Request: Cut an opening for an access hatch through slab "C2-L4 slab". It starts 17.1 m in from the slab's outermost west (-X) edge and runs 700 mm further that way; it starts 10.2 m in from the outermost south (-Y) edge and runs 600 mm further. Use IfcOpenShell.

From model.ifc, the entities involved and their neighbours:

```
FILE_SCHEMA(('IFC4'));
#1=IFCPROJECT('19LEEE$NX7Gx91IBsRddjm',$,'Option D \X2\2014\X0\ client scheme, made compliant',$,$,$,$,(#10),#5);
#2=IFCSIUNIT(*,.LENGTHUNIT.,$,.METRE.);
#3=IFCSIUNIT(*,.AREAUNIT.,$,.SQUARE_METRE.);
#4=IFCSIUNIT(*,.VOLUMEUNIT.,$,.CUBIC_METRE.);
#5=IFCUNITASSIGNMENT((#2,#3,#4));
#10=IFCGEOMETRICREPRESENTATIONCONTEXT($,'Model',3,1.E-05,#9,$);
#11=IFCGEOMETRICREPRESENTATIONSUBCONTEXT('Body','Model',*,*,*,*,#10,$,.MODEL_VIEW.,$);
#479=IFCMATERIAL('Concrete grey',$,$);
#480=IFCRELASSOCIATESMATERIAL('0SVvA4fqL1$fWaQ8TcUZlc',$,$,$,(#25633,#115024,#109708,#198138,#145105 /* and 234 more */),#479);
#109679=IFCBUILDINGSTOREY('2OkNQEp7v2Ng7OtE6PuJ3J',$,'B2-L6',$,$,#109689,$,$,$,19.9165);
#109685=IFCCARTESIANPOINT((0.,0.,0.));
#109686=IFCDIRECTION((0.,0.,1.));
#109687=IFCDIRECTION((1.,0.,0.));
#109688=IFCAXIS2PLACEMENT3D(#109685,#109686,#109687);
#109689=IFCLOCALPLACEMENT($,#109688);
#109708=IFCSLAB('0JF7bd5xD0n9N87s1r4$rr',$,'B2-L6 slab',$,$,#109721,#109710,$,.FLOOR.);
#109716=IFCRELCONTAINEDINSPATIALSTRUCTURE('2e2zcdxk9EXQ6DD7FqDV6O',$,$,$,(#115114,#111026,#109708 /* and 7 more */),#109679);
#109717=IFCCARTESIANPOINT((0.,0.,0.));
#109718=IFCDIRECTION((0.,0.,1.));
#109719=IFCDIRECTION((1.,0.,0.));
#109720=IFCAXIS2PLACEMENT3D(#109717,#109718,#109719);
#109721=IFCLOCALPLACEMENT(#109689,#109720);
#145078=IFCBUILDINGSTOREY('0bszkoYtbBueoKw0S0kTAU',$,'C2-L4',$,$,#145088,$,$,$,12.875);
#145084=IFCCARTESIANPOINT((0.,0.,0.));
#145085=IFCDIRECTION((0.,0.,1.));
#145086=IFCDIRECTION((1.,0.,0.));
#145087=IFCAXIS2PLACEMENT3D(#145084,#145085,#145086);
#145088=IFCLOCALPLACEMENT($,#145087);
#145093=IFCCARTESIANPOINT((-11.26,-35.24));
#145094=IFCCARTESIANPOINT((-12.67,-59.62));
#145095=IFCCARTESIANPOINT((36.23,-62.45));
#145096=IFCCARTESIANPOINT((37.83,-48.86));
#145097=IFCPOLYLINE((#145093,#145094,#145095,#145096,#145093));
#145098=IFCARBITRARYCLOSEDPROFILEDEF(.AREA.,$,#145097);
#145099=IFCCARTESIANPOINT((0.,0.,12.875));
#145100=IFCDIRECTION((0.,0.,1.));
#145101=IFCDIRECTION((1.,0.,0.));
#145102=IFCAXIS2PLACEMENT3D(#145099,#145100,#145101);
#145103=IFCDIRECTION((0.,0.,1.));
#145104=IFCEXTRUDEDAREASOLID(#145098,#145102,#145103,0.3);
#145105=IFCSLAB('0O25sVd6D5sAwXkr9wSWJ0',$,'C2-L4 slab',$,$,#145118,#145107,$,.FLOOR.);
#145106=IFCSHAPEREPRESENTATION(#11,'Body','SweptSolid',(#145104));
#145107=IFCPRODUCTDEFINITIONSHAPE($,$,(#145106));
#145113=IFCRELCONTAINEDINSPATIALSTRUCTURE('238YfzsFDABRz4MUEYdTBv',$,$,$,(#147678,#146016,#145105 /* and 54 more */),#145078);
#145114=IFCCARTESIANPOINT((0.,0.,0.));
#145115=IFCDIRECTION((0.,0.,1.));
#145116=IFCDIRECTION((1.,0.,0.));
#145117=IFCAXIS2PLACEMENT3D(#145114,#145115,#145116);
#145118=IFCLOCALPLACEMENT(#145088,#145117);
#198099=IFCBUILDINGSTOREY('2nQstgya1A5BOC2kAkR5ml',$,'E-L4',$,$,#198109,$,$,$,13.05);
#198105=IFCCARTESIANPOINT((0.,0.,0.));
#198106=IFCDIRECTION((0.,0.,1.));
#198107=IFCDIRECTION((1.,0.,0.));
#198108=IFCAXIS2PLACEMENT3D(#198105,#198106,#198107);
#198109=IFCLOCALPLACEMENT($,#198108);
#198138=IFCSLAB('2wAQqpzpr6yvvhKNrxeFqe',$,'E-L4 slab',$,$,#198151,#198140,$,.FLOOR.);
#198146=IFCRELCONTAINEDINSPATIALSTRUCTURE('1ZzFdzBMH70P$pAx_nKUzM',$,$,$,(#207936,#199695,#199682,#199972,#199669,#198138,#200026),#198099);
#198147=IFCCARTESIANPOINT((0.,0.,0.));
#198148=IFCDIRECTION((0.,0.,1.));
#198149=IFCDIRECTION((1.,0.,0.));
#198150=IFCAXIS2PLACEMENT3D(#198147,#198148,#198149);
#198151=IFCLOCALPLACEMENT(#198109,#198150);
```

```python
import numpy as np
import ifcopenshell
import ifcopenshell.api.feature
import ifcopenshell.api.geometry
import ifcopenshell.api.root
import ifcopenshell.geom
import ifcopenshell.util.placement
import ifcopenshell.util.representation
import ifcopenshell.util.shape
import ifcopenshell.util.unit

model = ifcopenshell.open("model.ifc")
unit_scale = ifcopenshell.util.unit.calculate_unit_scale(model)
settings = ifcopenshell.geom.settings()


def volume(element):
    """Net volume in cubic metres, openings subtracted."""
    shape = ifcopenshell.geom.create_shape(settings, element)
    return ifcopenshell.util.shape.get_volume(shape.geometry)


slab = model.by_guid("0O25sVd6D5sAwXkr9wSWJ0")
before = volume(slab)

# Extent in the slab's own axes, in metres. The edges named are its -X and -Y sides.
slab_shape = ifcopenshell.geom.create_shape(settings, slab)
vertices = ifcopenshell.util.shape.get_vertices(slab_shape.geometry)
x_min, y_min, bottom = vertices.min(axis=0)
top = vertices[:, 2].max()

opening = ifcopenshell.api.root.create_entity(model, ifc_class="IfcOpeningElement", name="Access hatch opening", predefined_type="OPENING")
context = ifcopenshell.util.representation.get_context(model, "Model", "Body", "MODEL_VIEW")
width, depth = 0.7, 0.6
outline = [(0.0, 0.0), (width, 0.0), (width, depth), (0.0, depth), (0.0, 0.0)]
# Overshoot both faces by 50 mm so the cut is clean.
shape = ifcopenshell.api.geometry.add_slab_representation(
    model, context=context, depth=top - bottom + 0.1, polyline=outline
)
ifcopenshell.api.geometry.assign_representation(model, product=opening, representation=shape)

matrix = ifcopenshell.util.placement.get_local_placement(slab.ObjectPlacement)
matrix[:, 3] = matrix @ np.append(np.array([x_min + 17.1, y_min + 10.2, bottom - 0.05]) / unit_scale, 1.0)
ifcopenshell.api.geometry.edit_object_placement(model, product=opening, matrix=matrix, is_si=False)
ifcopenshell.api.feature.add_feature(model, feature=opening, element=slab)

after = volume(slab)

print(f"slab volume {before:.3f} -> {after:.3f} m3")

model.write("model_rev.ifc")
```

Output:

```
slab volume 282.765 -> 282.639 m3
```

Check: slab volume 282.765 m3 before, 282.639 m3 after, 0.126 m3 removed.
